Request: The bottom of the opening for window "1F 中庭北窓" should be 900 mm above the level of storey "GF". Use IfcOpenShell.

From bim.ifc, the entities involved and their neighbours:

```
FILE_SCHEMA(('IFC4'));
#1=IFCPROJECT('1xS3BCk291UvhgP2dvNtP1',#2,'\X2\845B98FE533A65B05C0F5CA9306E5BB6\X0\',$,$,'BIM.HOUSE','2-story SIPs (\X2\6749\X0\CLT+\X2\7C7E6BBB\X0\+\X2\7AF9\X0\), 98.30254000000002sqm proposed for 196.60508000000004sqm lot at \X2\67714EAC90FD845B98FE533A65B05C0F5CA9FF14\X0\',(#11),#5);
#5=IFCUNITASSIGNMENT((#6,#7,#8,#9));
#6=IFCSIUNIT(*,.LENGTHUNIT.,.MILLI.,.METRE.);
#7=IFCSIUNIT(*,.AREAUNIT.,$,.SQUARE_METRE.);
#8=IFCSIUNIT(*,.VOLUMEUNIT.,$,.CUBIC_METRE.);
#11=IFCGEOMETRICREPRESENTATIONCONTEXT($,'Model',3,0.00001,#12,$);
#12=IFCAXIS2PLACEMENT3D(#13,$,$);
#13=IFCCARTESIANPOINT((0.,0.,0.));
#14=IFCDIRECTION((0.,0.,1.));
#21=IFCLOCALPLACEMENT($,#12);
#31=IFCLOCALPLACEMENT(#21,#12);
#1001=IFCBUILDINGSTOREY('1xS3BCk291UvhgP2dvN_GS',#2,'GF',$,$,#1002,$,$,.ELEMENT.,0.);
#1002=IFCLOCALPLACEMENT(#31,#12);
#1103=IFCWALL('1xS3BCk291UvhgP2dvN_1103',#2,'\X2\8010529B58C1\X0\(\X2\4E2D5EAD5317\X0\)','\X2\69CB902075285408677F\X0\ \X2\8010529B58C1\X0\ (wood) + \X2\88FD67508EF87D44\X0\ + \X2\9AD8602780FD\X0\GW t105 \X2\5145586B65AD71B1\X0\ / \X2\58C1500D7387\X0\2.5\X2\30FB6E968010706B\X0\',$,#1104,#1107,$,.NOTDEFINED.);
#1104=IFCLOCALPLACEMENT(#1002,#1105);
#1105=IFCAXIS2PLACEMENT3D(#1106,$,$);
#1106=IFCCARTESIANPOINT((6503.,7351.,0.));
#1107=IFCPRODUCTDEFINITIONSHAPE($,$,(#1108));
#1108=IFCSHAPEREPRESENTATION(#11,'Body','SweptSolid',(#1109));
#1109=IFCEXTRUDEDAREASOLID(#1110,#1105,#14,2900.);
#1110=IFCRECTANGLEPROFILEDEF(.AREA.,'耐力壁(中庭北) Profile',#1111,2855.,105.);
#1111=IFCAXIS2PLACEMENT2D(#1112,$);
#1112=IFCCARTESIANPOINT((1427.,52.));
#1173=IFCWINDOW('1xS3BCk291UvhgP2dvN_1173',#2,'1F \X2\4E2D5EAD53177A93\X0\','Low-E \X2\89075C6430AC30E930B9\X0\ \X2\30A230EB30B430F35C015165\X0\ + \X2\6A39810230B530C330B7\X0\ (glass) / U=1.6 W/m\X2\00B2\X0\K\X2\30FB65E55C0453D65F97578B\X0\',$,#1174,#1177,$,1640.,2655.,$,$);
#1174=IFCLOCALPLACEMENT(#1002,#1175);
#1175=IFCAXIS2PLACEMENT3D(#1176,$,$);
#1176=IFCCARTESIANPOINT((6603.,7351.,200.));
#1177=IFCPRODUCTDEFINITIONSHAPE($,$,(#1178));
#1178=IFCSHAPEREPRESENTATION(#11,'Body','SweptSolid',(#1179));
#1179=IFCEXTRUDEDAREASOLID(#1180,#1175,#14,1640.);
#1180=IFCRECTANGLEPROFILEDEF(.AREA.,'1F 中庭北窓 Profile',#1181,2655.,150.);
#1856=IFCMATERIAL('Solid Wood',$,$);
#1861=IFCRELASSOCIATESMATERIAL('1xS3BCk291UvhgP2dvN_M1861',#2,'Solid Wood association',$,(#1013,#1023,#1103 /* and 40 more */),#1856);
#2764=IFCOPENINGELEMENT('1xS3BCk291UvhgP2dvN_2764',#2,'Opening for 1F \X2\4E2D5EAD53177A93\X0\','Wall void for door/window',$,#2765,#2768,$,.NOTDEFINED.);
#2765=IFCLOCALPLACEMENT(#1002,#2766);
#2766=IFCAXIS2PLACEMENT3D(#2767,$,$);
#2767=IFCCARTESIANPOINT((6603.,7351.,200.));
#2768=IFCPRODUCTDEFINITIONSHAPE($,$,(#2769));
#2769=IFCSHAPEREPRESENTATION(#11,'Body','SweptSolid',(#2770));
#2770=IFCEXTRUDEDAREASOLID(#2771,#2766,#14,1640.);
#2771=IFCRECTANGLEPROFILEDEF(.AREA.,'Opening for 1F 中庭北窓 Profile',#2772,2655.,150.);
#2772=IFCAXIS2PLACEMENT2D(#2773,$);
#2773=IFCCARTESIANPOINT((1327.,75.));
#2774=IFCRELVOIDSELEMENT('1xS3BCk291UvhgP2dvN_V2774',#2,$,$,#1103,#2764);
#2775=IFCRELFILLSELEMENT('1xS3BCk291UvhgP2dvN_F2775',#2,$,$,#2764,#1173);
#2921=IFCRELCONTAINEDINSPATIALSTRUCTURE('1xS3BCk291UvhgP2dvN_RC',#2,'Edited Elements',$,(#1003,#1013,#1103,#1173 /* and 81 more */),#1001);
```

```python
import numpy as np
import ifcopenshell
import ifcopenshell.api.geometry
import ifcopenshell.geom
import ifcopenshell.util.element
import ifcopenshell.util.placement
import ifcopenshell.util.shape
import ifcopenshell.util.unit

model = ifcopenshell.open("bim.ifc")
unit_scale = ifcopenshell.util.unit.calculate_unit_scale(model)

window = model.by_guid("1xS3BCk291UvhgP2dvN_1173")
opening = window.FillsVoids[0].RelatingOpeningElement
storey = ifcopenshell.util.element.get_container(window, ifc_class="IfcBuildingStorey")
level = ifcopenshell.util.placement.get_local_placement(storey.ObjectPlacement)[2, 3]

# The opening's origin need not be at the sill, so measure its lowest point.
shape = ifcopenshell.geom.create_shape(ifcopenshell.geom.settings(), opening)
bottom = ifcopenshell.util.shape.get_shape_bottom_elevation(shape, shape.geometry) / unit_scale
dz = level + 0.9 / unit_scale - bottom

shift = np.array([0.0, 0.0, dz])
# The window is not placed relative to its opening, so move both.
for product in (opening, window):
    matrix = ifcopenshell.util.placement.get_local_placement(product.ObjectPlacement)
    matrix[:3, 3] += shift
    ifcopenshell.api.geometry.edit_object_placement(model, product=product, matrix=matrix, is_si=False)

print(f"moved by {dz * unit_scale:+.3f} m")

model.write("bim_updated.ifc")
```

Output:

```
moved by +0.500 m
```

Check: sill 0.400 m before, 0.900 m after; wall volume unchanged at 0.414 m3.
